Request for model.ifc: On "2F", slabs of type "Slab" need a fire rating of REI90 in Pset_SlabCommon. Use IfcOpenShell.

First a look at what the model holds.

```python
import ifcopenshell
import ifcopenshell.util.element

model = ifcopenshell.open("model.ifc")
print(model.schema)
storey = next(s for s in model.by_type("IfcBuildingStorey") if s.Name == "2F")
slabs = [e for e in ifcopenshell.util.element.get_decomposition(storey) if e.is_a("IfcSlab")]
seen = {}
for e in slabs:
    element_type = ifcopenshell.util.element.get_type(e)
    key = (element_type.Name if element_type != e and element_type else None, ifcopenshell.util.element.get_pset(e, "Pset_SlabCommon", "FireRating"))
    seen[key] = seen.get(key, 0) + 1
for (name, value), count in sorted(seen.items(), key=str):
    print(count, "x", name, "|", value)
```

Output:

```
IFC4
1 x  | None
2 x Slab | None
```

```python
import ifcopenshell
import ifcopenshell.api.pset
import ifcopenshell.util.element

model = ifcopenshell.open("model.ifc")

storey = next(s for s in model.by_type("IfcBuildingStorey") if s.Name == "2F")
slabs = [e for e in ifcopenshell.util.element.get_decomposition(storey) if e.is_a("IfcSlab")]

count = 0
for e in slabs:
    element_type = ifcopenshell.util.element.get_type(e)
    if element_type in (None, e) or element_type.Name != "Slab":
        continue
    # add_pset returns the element's existing set when there is one.
    pset = ifcopenshell.api.pset.add_pset(model, product=e, name="Pset_SlabCommon")
    ifcopenshell.api.pset.edit_pset(model, pset=pset, properties={"FireRating": "REI90"})
    count += 1

print(count, "slabs updated")

model.write("model_updated.ifc")
```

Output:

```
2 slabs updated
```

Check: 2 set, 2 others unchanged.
